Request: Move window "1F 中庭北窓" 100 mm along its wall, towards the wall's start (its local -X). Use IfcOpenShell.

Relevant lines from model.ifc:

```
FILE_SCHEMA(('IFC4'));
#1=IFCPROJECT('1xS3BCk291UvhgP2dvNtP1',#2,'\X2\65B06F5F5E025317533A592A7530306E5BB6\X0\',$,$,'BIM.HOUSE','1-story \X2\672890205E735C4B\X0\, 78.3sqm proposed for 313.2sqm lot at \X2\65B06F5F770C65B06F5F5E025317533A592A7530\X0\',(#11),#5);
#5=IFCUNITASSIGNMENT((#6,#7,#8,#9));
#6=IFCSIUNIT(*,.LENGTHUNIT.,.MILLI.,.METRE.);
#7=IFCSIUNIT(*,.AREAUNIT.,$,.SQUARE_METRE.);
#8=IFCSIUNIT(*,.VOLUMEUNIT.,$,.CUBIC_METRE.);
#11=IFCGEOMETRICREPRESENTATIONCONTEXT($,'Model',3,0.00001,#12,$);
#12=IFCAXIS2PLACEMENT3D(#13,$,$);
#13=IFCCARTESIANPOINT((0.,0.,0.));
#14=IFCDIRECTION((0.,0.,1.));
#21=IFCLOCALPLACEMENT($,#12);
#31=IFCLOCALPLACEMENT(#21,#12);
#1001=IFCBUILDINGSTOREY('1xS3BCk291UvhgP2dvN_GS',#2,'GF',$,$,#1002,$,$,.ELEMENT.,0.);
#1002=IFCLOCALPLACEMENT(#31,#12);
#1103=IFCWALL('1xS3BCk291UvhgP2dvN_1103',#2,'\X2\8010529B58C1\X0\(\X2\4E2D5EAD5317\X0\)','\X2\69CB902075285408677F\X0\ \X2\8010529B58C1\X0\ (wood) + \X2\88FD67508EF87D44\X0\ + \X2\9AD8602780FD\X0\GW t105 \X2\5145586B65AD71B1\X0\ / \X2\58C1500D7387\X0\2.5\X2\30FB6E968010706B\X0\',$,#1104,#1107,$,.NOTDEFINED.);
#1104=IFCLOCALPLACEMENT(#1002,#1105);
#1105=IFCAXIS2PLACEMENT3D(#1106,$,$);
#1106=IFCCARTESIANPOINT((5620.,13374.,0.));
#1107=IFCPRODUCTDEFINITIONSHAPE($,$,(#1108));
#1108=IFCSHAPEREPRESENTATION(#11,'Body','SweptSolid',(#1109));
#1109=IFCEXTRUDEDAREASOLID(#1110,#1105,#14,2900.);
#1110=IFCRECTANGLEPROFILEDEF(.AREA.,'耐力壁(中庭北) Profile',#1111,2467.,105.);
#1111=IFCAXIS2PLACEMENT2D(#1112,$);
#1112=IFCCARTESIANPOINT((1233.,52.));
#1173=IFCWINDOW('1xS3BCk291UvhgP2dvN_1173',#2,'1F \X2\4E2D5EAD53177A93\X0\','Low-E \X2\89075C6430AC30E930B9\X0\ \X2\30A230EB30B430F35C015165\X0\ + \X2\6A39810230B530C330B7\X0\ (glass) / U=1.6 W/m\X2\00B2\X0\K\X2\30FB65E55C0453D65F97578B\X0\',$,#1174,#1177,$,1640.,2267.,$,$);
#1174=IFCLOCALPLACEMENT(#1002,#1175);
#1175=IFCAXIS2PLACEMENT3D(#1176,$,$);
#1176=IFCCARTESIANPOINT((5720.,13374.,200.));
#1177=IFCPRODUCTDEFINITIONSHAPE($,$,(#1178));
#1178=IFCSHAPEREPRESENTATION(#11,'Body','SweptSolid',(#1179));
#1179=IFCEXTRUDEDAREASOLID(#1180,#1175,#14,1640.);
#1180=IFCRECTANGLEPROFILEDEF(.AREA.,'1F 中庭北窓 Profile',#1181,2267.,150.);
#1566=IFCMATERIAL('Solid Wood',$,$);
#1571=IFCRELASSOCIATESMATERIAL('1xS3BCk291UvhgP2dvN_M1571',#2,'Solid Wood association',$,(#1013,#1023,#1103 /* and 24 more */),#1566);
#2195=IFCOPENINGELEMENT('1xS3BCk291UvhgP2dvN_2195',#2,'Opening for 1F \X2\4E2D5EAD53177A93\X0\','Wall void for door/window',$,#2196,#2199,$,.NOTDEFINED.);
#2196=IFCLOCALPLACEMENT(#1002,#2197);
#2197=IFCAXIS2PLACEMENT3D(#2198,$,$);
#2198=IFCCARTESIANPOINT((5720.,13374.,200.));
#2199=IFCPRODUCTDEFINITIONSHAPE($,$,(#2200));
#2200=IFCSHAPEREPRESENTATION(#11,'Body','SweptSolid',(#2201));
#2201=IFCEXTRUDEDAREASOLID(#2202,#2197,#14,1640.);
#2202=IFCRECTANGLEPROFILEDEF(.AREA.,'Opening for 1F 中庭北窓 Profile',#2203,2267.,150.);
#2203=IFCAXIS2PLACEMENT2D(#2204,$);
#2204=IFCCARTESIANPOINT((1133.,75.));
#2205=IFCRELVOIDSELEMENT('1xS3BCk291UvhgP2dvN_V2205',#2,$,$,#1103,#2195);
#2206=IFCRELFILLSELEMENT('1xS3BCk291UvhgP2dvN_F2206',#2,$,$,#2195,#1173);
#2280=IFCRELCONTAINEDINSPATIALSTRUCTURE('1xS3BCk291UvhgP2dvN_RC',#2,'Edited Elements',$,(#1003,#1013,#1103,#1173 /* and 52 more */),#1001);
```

```python
import ifcopenshell
import ifcopenshell.api.geometry
import ifcopenshell.util.placement
import ifcopenshell.util.unit

model = ifcopenshell.open("model.ifc")
unit_scale = ifcopenshell.util.unit.calculate_unit_scale(model)

window = model.by_guid("1xS3BCk291UvhgP2dvN_1173")
opening = window.FillsVoids[0].RelatingOpeningElement
wall = opening.VoidsElements[0].RelatingBuildingElement

wall_matrix = ifcopenshell.util.placement.get_local_placement(wall.ObjectPlacement)
shift = wall_matrix[:3, 0] * -0.1 / unit_scale
before = ifcopenshell.util.placement.get_local_placement(window.ObjectPlacement)[:3, 3].copy()

# The window is not placed relative to its opening, so move both.
for product in (opening, window):
    matrix = ifcopenshell.util.placement.get_local_placement(product.ObjectPlacement)
    matrix[:3, 3] += shift
    ifcopenshell.api.geometry.edit_object_placement(model, product=product, matrix=matrix, is_si=False)

after = ifcopenshell.util.placement.get_local_placement(window.ObjectPlacement)[:3, 3]
print("window moved by", (after - before).round(3) + 0.0)

model.write("model_updated.ifc")
```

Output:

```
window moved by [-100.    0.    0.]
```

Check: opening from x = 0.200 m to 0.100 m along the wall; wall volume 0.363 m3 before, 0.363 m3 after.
